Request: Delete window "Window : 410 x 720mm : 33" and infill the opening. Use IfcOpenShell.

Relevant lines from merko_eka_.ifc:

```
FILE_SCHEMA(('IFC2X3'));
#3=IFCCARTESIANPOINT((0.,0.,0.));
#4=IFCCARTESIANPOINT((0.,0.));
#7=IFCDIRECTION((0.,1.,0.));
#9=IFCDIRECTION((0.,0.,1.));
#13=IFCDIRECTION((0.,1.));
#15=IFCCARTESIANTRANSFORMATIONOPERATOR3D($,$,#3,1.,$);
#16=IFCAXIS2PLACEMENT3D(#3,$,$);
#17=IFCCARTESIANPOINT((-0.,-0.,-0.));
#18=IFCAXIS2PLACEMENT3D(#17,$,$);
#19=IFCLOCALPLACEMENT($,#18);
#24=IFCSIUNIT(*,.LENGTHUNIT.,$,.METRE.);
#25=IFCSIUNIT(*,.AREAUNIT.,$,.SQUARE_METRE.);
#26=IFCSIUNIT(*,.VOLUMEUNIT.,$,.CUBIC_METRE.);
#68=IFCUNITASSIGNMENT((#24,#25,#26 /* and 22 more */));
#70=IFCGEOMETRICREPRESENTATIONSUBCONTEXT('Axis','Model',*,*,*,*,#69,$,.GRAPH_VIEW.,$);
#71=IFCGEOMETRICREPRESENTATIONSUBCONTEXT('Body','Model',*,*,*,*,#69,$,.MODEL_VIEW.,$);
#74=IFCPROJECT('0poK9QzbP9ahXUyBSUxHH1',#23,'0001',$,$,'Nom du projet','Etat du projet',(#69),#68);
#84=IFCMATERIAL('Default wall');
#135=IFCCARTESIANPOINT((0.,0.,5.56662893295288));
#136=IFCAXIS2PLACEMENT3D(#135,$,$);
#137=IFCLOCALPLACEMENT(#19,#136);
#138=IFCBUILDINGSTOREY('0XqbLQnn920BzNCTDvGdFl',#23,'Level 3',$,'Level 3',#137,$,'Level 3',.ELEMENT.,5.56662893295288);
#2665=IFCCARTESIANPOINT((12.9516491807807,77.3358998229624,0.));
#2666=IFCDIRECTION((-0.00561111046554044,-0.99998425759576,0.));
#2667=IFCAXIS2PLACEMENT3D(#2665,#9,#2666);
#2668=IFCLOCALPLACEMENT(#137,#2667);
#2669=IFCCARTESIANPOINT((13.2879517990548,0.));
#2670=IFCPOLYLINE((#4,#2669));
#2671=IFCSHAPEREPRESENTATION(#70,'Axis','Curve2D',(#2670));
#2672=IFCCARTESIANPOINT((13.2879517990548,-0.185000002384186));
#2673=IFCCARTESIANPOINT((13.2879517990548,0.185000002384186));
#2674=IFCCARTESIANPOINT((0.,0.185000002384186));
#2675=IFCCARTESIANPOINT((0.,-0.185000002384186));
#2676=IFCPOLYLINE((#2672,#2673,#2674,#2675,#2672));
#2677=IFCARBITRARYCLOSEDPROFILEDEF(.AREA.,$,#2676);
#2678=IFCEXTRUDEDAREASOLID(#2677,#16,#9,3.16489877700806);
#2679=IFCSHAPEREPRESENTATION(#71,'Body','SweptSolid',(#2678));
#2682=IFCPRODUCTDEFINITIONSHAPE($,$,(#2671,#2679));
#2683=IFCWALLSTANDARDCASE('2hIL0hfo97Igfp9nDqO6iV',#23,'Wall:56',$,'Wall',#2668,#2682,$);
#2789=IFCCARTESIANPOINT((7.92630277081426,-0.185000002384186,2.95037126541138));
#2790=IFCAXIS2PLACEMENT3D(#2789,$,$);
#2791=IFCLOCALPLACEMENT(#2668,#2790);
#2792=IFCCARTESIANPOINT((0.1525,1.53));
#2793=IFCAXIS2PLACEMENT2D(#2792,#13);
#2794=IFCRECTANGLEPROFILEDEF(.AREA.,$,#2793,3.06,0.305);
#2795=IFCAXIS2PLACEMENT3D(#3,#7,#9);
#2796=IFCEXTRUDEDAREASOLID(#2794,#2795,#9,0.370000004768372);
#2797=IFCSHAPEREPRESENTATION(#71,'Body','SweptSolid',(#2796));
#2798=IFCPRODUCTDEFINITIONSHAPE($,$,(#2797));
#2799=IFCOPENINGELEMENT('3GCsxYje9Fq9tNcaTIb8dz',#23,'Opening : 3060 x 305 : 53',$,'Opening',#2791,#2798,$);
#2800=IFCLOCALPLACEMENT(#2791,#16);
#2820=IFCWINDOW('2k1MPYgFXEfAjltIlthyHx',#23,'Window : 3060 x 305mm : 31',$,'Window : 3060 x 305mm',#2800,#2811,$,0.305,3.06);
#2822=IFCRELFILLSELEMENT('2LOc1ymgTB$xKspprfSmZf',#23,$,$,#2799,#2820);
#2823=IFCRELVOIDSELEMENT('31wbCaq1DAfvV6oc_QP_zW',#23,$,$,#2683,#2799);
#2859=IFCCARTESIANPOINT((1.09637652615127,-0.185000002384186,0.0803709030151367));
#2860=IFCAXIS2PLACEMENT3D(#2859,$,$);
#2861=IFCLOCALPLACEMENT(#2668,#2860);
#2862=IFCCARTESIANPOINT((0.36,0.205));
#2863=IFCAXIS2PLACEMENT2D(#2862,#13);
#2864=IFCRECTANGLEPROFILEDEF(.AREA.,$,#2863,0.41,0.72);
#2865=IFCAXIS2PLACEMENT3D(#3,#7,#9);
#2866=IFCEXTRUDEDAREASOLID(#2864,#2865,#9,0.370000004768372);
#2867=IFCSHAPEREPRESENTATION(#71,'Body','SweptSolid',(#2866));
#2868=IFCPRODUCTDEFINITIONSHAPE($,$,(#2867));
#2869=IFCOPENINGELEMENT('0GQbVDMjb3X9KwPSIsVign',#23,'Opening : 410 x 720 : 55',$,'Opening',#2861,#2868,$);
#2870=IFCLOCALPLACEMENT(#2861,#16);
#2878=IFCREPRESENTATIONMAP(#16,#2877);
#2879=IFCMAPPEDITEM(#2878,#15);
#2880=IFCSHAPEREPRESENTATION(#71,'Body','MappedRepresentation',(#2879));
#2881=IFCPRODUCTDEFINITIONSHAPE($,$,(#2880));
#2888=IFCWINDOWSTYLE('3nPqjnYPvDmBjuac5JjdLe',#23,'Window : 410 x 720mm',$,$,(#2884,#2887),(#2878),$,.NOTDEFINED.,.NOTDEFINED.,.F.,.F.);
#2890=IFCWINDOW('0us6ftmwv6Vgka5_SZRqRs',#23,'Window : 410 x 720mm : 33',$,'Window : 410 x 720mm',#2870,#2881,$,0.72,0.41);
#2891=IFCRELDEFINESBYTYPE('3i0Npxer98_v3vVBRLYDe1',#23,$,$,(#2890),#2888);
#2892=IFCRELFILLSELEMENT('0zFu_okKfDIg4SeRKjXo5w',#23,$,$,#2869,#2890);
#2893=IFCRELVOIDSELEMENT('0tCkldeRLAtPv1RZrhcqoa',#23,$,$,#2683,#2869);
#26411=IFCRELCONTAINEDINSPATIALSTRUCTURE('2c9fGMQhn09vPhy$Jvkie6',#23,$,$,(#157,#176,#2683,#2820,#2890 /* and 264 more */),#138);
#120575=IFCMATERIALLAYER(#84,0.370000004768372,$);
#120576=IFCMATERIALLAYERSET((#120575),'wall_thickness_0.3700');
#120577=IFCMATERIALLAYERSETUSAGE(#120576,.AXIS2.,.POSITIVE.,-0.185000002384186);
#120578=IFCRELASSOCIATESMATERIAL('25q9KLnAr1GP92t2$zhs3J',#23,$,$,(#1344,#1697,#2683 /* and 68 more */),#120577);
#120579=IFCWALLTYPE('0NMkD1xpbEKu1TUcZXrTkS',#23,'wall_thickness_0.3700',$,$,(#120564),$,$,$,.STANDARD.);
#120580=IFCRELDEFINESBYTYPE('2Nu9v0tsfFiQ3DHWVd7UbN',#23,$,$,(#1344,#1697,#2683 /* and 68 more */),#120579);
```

```python
import ifcopenshell
import ifcopenshell.api.feature
import ifcopenshell.api.root
import ifcopenshell.geom
import ifcopenshell.util.shape

model = ifcopenshell.open("merko_eka_.ifc")
settings = ifcopenshell.geom.settings()


def volume(element):
    """Net volume in cubic metres, openings subtracted."""
    shape = ifcopenshell.geom.create_shape(settings, element)
    return ifcopenshell.util.shape.get_volume(shape.geometry)


window = model.by_id(2890)
opening = window.FillsVoids[0].RelatingOpeningElement
wall = opening.VoidsElements[0].RelatingBuildingElement
before = volume(wall)

ifcopenshell.api.root.remove_product(model, product=window)
ifcopenshell.api.feature.remove_feature(model, feature=opening)

after = volume(wall)

print(f"wall volume {before:.3f} -> {after:.3f} m3")

model.write("merko_eka__rev.ifc")
```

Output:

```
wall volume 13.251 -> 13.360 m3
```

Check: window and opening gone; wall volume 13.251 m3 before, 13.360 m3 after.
